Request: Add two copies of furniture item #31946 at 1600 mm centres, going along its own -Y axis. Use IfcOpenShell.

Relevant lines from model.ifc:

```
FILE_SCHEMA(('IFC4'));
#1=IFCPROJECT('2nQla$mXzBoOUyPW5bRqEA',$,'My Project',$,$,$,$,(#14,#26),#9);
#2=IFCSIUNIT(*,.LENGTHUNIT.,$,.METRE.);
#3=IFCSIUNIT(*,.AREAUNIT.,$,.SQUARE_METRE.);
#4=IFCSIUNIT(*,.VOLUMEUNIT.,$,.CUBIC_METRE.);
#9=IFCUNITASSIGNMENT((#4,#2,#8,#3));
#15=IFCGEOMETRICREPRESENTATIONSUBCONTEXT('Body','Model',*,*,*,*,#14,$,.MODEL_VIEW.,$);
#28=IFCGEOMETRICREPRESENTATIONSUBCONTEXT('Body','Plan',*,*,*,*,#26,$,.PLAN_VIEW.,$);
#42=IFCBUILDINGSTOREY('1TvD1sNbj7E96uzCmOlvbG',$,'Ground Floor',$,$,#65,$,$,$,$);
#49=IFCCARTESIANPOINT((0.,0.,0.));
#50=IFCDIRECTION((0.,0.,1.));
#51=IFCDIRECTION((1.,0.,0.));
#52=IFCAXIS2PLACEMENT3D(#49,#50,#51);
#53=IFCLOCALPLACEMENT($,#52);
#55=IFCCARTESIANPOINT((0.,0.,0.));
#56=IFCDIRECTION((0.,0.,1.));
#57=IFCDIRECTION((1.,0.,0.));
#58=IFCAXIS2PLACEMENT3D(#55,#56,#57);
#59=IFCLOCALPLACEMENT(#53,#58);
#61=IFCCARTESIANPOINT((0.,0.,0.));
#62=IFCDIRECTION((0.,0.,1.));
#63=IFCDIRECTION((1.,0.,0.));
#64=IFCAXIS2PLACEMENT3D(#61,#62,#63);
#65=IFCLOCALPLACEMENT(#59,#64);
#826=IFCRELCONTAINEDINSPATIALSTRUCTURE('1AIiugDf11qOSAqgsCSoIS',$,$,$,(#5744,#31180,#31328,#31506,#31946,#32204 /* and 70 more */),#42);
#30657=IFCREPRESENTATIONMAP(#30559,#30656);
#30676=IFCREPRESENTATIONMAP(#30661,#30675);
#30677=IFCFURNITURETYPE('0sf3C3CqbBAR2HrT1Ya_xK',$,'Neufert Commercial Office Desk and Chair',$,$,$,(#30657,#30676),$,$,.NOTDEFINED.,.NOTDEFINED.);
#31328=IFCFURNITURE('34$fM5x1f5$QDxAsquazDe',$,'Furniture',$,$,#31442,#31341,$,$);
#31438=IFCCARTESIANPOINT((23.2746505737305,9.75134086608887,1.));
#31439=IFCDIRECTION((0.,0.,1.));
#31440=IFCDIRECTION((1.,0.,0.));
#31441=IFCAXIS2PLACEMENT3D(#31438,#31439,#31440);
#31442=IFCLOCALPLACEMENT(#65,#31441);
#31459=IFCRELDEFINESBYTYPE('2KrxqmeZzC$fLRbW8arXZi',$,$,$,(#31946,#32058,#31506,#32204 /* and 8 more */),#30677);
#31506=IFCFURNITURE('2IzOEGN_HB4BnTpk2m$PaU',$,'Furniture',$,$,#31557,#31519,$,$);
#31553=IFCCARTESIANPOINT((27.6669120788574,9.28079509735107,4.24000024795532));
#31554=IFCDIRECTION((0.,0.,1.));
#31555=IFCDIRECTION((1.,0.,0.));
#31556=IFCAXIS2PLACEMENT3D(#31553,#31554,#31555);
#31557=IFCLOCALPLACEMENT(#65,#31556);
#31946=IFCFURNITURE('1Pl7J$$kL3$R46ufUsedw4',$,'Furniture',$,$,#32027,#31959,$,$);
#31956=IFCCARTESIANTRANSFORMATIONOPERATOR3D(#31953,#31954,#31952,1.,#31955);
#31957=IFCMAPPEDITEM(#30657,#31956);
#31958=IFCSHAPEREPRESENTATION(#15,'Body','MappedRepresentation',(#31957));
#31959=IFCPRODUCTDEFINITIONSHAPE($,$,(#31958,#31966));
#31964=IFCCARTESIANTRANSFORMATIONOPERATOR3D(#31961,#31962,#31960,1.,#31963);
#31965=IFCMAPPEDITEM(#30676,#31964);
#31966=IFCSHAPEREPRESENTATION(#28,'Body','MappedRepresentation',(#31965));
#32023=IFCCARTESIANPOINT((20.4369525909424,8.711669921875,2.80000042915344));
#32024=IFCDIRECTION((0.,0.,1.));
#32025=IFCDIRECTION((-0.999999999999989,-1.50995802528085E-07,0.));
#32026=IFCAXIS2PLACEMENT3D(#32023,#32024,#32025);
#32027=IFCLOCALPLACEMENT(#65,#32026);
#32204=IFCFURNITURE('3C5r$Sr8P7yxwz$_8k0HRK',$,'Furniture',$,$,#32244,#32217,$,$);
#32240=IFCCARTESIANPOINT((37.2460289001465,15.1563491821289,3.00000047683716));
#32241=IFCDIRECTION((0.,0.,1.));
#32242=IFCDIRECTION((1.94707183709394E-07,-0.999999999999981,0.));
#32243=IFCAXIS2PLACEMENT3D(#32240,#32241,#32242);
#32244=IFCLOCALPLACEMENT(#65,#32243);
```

```python
import ifcopenshell
import ifcopenshell.api.geometry
import ifcopenshell.api.root
import ifcopenshell.util.element
import ifcopenshell.util.placement

model = ifcopenshell.open("model.ifc")

source = model.by_guid("1Pl7J$$kL3$R46ufUsedw4")
base = ifcopenshell.util.placement.get_local_placement(source.ObjectPlacement)
step = -base[:3, 1] * 1.6

for i in range(1, 3):
    copy = ifcopenshell.api.root.copy_class(model, product=source)
    copy.Representation = ifcopenshell.util.element.copy_deep(
        model, source.Representation, exclude=["IfcGeometricRepresentationContext", "IfcRepresentationMap"]
    )
    matrix = base.copy()
    matrix[:3, 3] += i * step
    print("added at", matrix[:3, 3].round(3) + 0.0)
    ifcopenshell.api.geometry.edit_object_placement(model, product=copy, matrix=matrix, is_si=False)

model.write("model_v2.ifc")
```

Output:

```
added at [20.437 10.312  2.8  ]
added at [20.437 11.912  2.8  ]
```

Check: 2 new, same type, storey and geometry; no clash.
